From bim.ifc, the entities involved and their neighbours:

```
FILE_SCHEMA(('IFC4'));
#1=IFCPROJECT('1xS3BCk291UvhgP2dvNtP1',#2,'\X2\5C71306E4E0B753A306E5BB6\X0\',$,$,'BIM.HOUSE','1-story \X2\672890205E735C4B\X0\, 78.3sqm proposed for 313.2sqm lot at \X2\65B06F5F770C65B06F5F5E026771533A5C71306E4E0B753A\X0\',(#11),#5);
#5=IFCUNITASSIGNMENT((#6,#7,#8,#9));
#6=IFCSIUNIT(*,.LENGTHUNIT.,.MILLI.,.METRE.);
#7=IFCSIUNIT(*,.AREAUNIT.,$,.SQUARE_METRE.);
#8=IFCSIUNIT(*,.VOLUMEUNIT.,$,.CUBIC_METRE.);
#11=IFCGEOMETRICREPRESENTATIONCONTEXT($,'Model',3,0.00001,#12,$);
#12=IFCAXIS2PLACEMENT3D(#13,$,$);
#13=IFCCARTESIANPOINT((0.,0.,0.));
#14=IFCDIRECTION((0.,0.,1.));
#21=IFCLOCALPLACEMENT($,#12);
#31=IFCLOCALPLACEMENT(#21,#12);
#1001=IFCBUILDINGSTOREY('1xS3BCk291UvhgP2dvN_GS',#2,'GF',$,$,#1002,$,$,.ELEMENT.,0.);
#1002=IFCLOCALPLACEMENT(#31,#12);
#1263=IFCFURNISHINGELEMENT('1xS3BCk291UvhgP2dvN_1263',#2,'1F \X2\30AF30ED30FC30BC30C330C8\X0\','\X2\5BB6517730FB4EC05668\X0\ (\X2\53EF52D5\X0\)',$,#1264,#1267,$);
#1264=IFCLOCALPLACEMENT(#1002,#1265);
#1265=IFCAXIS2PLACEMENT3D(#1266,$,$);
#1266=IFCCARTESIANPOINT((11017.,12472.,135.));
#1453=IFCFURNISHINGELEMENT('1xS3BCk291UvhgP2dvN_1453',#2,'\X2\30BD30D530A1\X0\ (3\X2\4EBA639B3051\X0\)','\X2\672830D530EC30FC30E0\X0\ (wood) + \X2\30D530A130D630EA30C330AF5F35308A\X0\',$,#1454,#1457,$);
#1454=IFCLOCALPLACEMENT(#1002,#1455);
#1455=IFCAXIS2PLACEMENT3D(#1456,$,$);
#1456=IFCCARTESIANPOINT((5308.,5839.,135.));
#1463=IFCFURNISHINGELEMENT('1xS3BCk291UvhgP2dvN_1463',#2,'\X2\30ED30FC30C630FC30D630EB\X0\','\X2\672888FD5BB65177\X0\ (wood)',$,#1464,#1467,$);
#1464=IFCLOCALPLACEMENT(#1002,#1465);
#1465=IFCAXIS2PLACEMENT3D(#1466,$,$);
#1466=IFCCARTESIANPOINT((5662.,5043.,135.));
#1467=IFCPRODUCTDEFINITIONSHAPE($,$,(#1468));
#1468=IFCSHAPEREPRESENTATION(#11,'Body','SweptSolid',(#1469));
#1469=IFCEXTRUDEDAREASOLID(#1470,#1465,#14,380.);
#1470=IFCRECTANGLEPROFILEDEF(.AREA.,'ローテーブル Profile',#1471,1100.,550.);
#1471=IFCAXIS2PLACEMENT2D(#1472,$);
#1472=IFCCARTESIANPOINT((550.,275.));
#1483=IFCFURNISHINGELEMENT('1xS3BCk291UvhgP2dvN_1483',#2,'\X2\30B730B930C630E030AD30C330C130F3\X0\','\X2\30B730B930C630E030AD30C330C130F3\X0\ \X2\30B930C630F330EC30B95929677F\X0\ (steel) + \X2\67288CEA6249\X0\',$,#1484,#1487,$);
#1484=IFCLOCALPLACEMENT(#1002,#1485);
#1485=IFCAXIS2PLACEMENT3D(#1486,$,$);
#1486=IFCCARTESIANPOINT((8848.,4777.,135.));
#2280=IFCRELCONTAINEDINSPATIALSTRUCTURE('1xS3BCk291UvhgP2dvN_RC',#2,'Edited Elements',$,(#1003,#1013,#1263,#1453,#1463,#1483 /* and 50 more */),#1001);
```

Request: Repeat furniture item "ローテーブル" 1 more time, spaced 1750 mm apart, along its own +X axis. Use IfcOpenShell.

```python
import ifcopenshell
import ifcopenshell.api.geometry
import ifcopenshell.api.root
import ifcopenshell.util.element
import ifcopenshell.util.placement
import ifcopenshell.util.unit

model = ifcopenshell.open("bim.ifc")
unit_scale = ifcopenshell.util.unit.calculate_unit_scale(model)


def reuse_history(source, copy):
    """copy_class also copies each property set's owner history, people and application; keep the originals."""
    for rel in copy.IsDefinedBy:
        if rel.is_a("IfcRelDefinesByProperties") and (history := rel.RelatingPropertyDefinition.OwnerHistory):
            rel.RelatingPropertyDefinition.OwnerHistory = source.OwnerHistory
            ifcopenshell.util.element.remove_deep2(model, history)


source = model.by_id(1463)
base = ifcopenshell.util.placement.get_local_placement(source.ObjectPlacement)
step = base[:3, 0] * 1.75 / unit_scale

for i in range(1, 2):
    copy = ifcopenshell.api.root.copy_class(model, product=source)
    copy.Representation = ifcopenshell.util.element.copy_deep(
        model, source.Representation, exclude=["IfcGeometricRepresentationContext", "IfcRepresentationMap"]
    )
    reuse_history(source, copy)
    matrix = base.copy()
    matrix[:3, 3] += i * step
    print("added at", matrix[:3, 3].round(3) + 0.0)
    ifcopenshell.api.geometry.edit_object_placement(model, product=copy, matrix=matrix, is_si=False)

model.write("bim_updated.ifc")
```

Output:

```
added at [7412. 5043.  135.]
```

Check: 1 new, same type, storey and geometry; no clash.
